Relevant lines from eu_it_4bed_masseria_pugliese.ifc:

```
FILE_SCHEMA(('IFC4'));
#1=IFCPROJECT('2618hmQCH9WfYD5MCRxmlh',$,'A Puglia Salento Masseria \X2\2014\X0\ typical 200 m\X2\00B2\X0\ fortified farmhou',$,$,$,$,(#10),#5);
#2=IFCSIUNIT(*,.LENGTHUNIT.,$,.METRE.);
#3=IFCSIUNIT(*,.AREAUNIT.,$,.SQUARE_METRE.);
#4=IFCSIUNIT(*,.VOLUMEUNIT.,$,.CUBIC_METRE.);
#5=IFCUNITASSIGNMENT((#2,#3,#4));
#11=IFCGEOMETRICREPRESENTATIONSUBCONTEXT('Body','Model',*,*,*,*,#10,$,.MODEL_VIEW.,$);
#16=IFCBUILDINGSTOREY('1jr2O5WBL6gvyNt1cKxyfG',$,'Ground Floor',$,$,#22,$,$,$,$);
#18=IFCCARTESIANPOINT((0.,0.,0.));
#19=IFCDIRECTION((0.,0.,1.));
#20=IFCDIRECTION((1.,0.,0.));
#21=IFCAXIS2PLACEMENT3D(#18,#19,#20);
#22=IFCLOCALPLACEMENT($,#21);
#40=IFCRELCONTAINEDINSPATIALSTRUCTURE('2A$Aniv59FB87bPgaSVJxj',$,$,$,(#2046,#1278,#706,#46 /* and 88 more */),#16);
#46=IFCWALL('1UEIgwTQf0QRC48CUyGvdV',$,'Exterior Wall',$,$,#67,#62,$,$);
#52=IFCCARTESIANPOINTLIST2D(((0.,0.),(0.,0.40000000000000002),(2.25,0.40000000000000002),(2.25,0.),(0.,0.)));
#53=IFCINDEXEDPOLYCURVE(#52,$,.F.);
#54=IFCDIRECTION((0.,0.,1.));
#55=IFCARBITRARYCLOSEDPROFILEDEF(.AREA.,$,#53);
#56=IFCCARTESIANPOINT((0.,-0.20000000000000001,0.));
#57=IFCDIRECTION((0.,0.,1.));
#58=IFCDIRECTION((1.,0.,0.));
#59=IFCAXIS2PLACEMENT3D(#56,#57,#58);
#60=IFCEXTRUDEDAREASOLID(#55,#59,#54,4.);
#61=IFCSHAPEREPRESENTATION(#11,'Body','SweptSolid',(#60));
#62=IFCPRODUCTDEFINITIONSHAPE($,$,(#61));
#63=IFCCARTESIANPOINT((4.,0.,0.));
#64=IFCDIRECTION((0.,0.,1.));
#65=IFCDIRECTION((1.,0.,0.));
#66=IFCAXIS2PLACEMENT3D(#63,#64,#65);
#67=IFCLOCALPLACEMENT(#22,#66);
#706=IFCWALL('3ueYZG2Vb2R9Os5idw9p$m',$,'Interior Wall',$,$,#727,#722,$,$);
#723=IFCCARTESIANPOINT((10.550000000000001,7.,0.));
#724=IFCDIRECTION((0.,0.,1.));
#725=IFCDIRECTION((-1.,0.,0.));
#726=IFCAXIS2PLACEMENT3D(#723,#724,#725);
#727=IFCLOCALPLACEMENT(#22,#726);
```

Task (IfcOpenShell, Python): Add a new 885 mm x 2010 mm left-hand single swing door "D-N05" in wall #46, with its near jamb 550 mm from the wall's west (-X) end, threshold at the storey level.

```python
import numpy as np
import ifcopenshell
import ifcopenshell.api.feature
import ifcopenshell.api.geometry
import ifcopenshell.api.root
import ifcopenshell.api.spatial
import ifcopenshell.geom
import ifcopenshell.util.element
import ifcopenshell.util.placement
import ifcopenshell.util.representation
import ifcopenshell.util.shape
import ifcopenshell.util.unit

model = ifcopenshell.open("eu_it_4bed_masseria_pugliese.ifc")
unit_scale = ifcopenshell.util.unit.calculate_unit_scale(model)
settings = ifcopenshell.geom.settings()


def volume(element):
    """Net volume in cubic metres, openings subtracted."""
    shape = ifcopenshell.geom.create_shape(settings, element)
    return ifcopenshell.util.shape.get_volume(shape.geometry)


wall = model.by_id(46)
storey = ifcopenshell.util.element.get_container(wall, ifc_class="IfcBuildingStorey")
context = ifcopenshell.util.representation.get_context(model, "Model", "Body", "MODEL_VIEW")
before = volume(wall)

width, height, from_end, sill = 0.885, 2.01, 0.55, 0.0  # metres

# The wall runs along its own X axis, and the end named is its -X end.
wall_shape = ifcopenshell.geom.create_shape(settings, wall)
x, y, z = ifcopenshell.util.shape.get_vertices(wall_shape.geometry).T
start = x.min() + from_end
face, thickness = float(y.min()), float(y.max() - y.min())
wall_matrix = ifcopenshell.util.placement.get_local_placement(wall.ObjectPlacement)
level = ifcopenshell.util.placement.get_local_placement(storey.ObjectPlacement)[2, 3]


def in_wall(x, y):
    """Placement at x, y metres in the wall's axes, at sill height."""
    matrix = wall_matrix.copy()
    matrix[:, 3] = wall_matrix @ np.array([x / unit_scale, y / unit_scale, 0.0, 1.0])
    matrix[2, 3] = level + sill / unit_scale
    return matrix


# Opening: a box that overshoots both wall faces by 50 mm.
opening = ifcopenshell.api.root.create_entity(model, ifc_class="IfcOpeningElement", predefined_type="OPENING")
box = ifcopenshell.api.geometry.add_wall_representation(
    model, context=context, length=width, height=height, thickness=thickness + 0.1
)
ifcopenshell.api.geometry.assign_representation(model, product=opening, representation=box)
ifcopenshell.api.geometry.edit_object_placement(model, product=opening, matrix=in_wall(start, face - 0.05), is_si=False)
ifcopenshell.api.feature.add_feature(model, feature=opening, element=wall)

door = ifcopenshell.api.root.create_entity(model, ifc_class="IfcDoor", name="D-N05", predefined_type="DOOR")
door.OverallWidth, door.OverallHeight = width / unit_scale, height / unit_scale
door.OperationType = "SINGLE_SWING_LEFT"
body = ifcopenshell.api.geometry.add_door_representation(
    model,
    context=context,
    overall_width=door.OverallWidth,
    overall_height=door.OverallHeight,
    operation_type="SINGLE_SWING_LEFT",
    lining_properties={"LiningDepth": thickness / unit_scale, "ThresholdDepth": thickness / unit_scale},
)
ifcopenshell.api.geometry.assign_representation(model, product=door, representation=body)
ifcopenshell.api.spatial.assign_container(model, products=[door], relating_structure=storey)
ifcopenshell.api.feature.add_filling(model, opening=opening, element=door)

# The lining spans the wall, so the door starts at the wall face.
ifcopenshell.api.geometry.edit_object_placement(model, product=door, matrix=in_wall(start, face), is_si=False)

after = volume(wall)

print(f"wall volume {before:.3f} -> {after:.3f} m3")

model.write("eu_it_4bed_masseria_pugliese_v2.ifc")
```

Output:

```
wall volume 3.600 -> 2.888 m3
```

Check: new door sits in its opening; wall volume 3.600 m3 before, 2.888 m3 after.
